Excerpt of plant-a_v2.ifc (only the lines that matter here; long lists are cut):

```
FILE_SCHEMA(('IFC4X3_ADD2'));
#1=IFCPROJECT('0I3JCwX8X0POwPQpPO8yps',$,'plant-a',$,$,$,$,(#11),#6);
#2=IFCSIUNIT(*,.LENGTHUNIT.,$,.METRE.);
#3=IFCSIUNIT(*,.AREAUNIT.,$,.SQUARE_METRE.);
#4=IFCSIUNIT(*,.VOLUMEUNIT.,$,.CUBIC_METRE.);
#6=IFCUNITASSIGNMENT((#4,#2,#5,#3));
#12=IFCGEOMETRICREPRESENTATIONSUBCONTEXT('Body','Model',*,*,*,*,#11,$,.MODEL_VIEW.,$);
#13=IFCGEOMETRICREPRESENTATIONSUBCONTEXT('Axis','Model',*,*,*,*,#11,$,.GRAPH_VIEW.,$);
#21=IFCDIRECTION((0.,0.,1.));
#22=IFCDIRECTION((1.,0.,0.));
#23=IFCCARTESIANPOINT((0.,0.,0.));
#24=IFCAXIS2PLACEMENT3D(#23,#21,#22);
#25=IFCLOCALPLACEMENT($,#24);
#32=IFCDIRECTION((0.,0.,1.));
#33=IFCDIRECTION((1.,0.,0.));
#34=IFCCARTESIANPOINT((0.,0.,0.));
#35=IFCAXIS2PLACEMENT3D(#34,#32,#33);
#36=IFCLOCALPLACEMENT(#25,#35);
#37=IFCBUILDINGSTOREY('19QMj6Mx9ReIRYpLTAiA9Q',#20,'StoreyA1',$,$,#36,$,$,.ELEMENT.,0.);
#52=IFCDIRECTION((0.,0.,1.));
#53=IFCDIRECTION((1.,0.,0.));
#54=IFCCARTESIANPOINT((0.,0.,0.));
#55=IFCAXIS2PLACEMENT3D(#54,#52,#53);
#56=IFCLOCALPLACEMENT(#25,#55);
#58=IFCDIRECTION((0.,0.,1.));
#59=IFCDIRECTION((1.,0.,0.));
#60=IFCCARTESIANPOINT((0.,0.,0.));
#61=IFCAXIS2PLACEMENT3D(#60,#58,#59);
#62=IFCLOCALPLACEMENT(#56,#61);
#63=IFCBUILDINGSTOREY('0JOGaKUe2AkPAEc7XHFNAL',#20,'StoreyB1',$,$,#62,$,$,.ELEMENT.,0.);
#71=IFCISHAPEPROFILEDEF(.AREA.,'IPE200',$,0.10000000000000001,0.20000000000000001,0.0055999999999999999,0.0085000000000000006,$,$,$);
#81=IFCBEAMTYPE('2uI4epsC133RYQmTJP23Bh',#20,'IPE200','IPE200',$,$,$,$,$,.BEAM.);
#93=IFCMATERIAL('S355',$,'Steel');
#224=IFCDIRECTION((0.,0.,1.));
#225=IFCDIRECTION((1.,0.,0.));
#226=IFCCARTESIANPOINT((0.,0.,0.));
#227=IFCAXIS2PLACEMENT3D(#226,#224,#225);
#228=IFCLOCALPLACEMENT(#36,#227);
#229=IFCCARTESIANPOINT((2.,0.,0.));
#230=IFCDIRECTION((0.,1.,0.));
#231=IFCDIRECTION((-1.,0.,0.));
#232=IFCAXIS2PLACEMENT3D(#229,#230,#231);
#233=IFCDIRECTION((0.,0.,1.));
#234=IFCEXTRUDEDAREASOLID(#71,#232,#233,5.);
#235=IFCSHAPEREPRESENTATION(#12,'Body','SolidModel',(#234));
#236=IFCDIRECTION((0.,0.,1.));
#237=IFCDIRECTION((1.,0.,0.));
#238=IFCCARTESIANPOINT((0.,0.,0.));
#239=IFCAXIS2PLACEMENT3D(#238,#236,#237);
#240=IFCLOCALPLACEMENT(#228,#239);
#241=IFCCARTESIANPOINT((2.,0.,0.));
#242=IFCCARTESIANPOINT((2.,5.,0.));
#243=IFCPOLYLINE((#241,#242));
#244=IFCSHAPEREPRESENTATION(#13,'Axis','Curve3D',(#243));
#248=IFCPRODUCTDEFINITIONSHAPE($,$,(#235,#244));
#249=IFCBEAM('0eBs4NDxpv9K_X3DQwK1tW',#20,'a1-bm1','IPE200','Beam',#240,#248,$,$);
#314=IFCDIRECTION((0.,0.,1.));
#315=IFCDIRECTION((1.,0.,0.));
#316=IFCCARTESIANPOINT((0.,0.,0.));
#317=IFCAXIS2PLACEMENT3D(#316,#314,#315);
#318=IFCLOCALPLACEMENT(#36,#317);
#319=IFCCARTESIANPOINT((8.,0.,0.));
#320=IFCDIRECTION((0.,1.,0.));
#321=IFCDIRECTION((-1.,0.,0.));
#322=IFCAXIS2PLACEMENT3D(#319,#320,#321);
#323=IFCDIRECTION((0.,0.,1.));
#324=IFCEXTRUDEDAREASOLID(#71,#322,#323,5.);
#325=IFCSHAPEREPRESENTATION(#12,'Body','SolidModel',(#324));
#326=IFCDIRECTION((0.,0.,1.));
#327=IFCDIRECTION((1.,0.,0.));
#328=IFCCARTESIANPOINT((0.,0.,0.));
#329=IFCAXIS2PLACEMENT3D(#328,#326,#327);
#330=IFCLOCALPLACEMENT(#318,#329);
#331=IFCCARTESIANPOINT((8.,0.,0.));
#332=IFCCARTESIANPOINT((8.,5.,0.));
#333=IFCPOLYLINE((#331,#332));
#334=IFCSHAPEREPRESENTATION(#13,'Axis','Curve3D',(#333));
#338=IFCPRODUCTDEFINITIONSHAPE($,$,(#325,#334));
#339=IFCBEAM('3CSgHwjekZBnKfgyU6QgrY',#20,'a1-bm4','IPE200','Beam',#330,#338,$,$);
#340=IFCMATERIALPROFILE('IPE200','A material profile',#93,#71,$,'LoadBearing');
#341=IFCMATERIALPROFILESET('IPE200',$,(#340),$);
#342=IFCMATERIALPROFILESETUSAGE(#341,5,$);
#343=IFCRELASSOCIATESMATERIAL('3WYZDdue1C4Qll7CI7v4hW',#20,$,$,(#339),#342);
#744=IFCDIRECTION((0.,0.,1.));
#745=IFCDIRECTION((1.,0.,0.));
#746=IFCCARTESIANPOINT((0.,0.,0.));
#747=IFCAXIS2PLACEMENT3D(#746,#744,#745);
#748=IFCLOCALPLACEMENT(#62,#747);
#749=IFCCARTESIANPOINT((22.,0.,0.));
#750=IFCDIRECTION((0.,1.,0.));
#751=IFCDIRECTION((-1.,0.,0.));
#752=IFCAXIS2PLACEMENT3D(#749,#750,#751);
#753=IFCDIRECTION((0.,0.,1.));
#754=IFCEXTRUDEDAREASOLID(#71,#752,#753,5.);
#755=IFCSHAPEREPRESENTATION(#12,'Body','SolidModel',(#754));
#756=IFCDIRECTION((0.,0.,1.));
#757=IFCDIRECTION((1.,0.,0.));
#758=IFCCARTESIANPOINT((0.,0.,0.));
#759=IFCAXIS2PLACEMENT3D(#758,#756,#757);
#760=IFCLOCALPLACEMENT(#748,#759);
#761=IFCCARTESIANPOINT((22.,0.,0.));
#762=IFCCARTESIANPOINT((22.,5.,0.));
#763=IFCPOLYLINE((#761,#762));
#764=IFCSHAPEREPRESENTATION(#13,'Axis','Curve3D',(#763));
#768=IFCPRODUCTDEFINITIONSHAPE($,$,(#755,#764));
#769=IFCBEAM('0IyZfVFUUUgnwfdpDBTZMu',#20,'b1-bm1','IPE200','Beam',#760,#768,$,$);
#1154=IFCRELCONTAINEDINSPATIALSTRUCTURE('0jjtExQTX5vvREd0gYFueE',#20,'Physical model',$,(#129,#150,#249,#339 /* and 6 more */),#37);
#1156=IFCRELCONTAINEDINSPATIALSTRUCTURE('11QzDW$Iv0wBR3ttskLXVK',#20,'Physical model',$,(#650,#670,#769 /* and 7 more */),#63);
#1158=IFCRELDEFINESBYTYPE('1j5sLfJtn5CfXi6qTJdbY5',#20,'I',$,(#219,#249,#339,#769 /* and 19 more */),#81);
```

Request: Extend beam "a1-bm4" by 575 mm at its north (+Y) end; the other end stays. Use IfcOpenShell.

```python
import numpy as np
import ifcopenshell
import ifcopenshell.util.representation

model = ifcopenshell.open("plant-a_v2.ifc")

member = model.by_id(339)
change = 0.575

# The extrusion runs towards the end named, so only its depth changes.
body = ifcopenshell.util.representation.get_representation(member, "Model", "Body")
solid = body.Items[0]
old_length = solid.Depth
solid.Depth += change

# Move the axis end point with it.
axis = next(r for r in member.Representation.Representations if r.RepresentationIdentifier == "Axis").Items[0]
start, end = (np.array(p.Coordinates) for p in axis.Points)
end = end + (end - start) / np.linalg.norm(end - start) * change
point = model.createIfcCartesianPoint(end.tolist())
axis.Points = [axis.Points[0], point]

print(f"length {old_length:g} -> {solid.Depth:g}")

model.write("plant-a_v2_rev.ifc")
```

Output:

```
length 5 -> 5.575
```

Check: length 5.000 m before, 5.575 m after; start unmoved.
